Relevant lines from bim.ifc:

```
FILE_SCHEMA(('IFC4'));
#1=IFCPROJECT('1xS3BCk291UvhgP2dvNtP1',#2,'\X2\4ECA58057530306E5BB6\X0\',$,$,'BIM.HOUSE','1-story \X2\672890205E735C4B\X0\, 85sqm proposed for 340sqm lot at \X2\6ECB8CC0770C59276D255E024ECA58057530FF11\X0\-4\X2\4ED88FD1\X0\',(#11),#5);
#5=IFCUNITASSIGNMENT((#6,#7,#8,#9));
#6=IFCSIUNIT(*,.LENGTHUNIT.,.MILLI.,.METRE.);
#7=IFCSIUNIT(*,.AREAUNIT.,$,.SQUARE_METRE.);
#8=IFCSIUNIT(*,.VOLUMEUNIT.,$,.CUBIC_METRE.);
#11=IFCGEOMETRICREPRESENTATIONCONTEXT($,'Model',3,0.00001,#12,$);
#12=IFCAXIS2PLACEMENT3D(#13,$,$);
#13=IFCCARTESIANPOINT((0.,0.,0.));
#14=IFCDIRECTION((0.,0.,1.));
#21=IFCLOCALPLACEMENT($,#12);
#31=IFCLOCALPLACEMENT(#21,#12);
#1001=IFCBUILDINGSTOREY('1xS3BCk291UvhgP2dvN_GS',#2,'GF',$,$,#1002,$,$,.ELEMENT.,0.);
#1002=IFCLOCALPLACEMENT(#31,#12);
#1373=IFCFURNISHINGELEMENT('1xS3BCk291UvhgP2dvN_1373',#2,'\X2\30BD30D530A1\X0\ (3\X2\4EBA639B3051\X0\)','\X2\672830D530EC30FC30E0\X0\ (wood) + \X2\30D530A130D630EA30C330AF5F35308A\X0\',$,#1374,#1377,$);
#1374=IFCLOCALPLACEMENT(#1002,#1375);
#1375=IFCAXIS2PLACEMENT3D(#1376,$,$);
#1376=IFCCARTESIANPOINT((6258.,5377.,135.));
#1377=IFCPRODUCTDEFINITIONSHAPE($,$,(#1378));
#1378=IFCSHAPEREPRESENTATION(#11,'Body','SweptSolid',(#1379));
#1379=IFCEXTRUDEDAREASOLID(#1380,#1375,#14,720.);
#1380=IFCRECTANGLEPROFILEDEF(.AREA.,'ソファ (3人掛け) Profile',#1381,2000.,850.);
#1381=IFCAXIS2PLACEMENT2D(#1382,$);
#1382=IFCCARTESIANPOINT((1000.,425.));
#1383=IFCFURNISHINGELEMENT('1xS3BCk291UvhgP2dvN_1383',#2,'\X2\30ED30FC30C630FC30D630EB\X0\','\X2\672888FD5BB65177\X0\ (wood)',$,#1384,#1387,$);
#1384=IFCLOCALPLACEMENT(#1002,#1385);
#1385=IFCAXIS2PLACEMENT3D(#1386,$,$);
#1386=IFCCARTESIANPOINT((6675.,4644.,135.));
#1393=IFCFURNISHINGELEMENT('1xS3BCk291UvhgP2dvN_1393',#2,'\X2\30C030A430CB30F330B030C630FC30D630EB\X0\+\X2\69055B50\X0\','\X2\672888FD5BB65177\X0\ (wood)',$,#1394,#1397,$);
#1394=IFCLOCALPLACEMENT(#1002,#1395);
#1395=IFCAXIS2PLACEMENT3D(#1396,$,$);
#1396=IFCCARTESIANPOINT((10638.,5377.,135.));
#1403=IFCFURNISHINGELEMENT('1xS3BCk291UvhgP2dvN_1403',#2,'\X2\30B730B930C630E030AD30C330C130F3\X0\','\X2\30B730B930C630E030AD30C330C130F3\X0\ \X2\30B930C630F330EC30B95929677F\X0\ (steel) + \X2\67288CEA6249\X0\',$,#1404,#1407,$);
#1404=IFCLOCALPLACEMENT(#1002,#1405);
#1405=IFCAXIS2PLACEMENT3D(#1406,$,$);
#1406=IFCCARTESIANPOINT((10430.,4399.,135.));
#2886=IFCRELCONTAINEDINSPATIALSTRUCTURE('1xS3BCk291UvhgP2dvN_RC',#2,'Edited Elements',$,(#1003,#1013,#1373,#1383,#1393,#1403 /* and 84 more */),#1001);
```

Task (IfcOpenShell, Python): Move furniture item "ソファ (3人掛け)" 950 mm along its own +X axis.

```python
import ifcopenshell
import ifcopenshell.api.geometry
import ifcopenshell.util.placement
import ifcopenshell.util.unit

model = ifcopenshell.open("bim.ifc")
unit_scale = ifcopenshell.util.unit.calculate_unit_scale(model)

item = model.by_id(1373)
matrix = ifcopenshell.util.placement.get_local_placement(item.ObjectPlacement)
matrix[:3, 3] += matrix[:3, 0] * 0.95 / unit_scale
ifcopenshell.api.geometry.edit_object_placement(model, product=item, matrix=matrix, is_si=False)

print(ifcopenshell.util.placement.get_local_placement(item.ObjectPlacement).round(3) + 0.0)

model.write("bim_updated.ifc")
```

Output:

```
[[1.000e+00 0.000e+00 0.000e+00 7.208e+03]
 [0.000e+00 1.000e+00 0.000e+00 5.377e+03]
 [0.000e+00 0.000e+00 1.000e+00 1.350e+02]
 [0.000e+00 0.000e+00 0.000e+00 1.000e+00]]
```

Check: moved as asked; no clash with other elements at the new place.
